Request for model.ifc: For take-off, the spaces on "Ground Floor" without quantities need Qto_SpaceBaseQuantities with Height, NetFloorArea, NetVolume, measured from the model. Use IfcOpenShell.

First a look at what the model holds.

```python
import ifcopenshell
import ifcopenshell.util.element
import ifcopenshell.util.unit

model = ifcopenshell.open("model.ifc")
print(model.schema)
for unit_type in ("LENGTHUNIT", "AREAUNIT", "VOLUMEUNIT"):
    print(unit_type, ifcopenshell.util.unit.calculate_unit_scale(model, unit_type))
storey = next(s for s in model.by_type("IfcBuildingStorey") if s.Name == "Ground Floor")
spaces = [e for e in ifcopenshell.util.element.get_decomposition(storey) if e.is_a("IfcSpace")]
for e in sorted(spaces, key=lambda e: e.id()):
    print(e.id(), e.is_a(), e.Name, list(ifcopenshell.util.element.get_psets(e, qtos_only=True)), sep=" | ")
```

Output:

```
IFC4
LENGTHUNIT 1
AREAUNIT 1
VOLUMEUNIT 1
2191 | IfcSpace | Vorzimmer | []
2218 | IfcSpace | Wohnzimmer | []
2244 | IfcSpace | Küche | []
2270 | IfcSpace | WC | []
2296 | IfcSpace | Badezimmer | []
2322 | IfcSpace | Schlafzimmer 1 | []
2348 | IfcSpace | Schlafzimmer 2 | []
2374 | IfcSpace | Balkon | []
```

```python
import ifcopenshell
import ifcopenshell.api.pset
import ifcopenshell.geom
import ifcopenshell.util.element
import ifcopenshell.util.shape
import ifcopenshell.util.unit

model = ifcopenshell.open("model.ifc")
unit_scale = ifcopenshell.util.unit.calculate_unit_scale(model)
area_scale = ifcopenshell.util.unit.calculate_unit_scale(model, "AREAUNIT")
volume_scale = ifcopenshell.util.unit.calculate_unit_scale(model, "VOLUMEUNIT")
settings = ifcopenshell.geom.settings()

storey = next(s for s in model.by_type("IfcBuildingStorey") if s.Name == "Ground Floor")
spaces = [e for e in ifcopenshell.util.element.get_decomposition(storey) if e.is_a("IfcSpace")]

for e in sorted(spaces, key=lambda e: e.id()):
    if ifcopenshell.util.element.get_psets(e, qtos_only=True, should_inherit=False):
        continue
    # Geometry comes back in metres, in the element's own axes.
    shape = ifcopenshell.geom.create_shape(settings, e)
    values = {
        "Height": ifcopenshell.util.shape.get_z(shape.geometry) / unit_scale,
        "NetFloorArea": ifcopenshell.util.shape.get_footprint_area(shape.geometry) / area_scale,
        "NetVolume": ifcopenshell.util.shape.get_volume(shape.geometry) / volume_scale,
    }
    qto = ifcopenshell.api.pset.add_qto(model, product=e, name="Qto_SpaceBaseQuantities")
    ifcopenshell.api.pset.edit_qto(model, qto=qto, properties=values)
    print(e.id(), {k: round(v, 3) for k, v in values.items()})

model.write("model_updated.ifc")
```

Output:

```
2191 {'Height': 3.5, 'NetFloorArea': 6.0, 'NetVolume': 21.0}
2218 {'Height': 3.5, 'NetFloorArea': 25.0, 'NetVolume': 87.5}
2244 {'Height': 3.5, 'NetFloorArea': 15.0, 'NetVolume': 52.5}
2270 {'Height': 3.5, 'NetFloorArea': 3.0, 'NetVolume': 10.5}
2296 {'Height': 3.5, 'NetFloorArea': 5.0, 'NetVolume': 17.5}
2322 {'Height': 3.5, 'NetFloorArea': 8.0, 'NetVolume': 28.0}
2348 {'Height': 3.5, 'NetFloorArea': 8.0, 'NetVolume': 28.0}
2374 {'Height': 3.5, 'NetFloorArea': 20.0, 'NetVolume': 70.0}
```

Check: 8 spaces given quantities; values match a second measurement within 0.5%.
